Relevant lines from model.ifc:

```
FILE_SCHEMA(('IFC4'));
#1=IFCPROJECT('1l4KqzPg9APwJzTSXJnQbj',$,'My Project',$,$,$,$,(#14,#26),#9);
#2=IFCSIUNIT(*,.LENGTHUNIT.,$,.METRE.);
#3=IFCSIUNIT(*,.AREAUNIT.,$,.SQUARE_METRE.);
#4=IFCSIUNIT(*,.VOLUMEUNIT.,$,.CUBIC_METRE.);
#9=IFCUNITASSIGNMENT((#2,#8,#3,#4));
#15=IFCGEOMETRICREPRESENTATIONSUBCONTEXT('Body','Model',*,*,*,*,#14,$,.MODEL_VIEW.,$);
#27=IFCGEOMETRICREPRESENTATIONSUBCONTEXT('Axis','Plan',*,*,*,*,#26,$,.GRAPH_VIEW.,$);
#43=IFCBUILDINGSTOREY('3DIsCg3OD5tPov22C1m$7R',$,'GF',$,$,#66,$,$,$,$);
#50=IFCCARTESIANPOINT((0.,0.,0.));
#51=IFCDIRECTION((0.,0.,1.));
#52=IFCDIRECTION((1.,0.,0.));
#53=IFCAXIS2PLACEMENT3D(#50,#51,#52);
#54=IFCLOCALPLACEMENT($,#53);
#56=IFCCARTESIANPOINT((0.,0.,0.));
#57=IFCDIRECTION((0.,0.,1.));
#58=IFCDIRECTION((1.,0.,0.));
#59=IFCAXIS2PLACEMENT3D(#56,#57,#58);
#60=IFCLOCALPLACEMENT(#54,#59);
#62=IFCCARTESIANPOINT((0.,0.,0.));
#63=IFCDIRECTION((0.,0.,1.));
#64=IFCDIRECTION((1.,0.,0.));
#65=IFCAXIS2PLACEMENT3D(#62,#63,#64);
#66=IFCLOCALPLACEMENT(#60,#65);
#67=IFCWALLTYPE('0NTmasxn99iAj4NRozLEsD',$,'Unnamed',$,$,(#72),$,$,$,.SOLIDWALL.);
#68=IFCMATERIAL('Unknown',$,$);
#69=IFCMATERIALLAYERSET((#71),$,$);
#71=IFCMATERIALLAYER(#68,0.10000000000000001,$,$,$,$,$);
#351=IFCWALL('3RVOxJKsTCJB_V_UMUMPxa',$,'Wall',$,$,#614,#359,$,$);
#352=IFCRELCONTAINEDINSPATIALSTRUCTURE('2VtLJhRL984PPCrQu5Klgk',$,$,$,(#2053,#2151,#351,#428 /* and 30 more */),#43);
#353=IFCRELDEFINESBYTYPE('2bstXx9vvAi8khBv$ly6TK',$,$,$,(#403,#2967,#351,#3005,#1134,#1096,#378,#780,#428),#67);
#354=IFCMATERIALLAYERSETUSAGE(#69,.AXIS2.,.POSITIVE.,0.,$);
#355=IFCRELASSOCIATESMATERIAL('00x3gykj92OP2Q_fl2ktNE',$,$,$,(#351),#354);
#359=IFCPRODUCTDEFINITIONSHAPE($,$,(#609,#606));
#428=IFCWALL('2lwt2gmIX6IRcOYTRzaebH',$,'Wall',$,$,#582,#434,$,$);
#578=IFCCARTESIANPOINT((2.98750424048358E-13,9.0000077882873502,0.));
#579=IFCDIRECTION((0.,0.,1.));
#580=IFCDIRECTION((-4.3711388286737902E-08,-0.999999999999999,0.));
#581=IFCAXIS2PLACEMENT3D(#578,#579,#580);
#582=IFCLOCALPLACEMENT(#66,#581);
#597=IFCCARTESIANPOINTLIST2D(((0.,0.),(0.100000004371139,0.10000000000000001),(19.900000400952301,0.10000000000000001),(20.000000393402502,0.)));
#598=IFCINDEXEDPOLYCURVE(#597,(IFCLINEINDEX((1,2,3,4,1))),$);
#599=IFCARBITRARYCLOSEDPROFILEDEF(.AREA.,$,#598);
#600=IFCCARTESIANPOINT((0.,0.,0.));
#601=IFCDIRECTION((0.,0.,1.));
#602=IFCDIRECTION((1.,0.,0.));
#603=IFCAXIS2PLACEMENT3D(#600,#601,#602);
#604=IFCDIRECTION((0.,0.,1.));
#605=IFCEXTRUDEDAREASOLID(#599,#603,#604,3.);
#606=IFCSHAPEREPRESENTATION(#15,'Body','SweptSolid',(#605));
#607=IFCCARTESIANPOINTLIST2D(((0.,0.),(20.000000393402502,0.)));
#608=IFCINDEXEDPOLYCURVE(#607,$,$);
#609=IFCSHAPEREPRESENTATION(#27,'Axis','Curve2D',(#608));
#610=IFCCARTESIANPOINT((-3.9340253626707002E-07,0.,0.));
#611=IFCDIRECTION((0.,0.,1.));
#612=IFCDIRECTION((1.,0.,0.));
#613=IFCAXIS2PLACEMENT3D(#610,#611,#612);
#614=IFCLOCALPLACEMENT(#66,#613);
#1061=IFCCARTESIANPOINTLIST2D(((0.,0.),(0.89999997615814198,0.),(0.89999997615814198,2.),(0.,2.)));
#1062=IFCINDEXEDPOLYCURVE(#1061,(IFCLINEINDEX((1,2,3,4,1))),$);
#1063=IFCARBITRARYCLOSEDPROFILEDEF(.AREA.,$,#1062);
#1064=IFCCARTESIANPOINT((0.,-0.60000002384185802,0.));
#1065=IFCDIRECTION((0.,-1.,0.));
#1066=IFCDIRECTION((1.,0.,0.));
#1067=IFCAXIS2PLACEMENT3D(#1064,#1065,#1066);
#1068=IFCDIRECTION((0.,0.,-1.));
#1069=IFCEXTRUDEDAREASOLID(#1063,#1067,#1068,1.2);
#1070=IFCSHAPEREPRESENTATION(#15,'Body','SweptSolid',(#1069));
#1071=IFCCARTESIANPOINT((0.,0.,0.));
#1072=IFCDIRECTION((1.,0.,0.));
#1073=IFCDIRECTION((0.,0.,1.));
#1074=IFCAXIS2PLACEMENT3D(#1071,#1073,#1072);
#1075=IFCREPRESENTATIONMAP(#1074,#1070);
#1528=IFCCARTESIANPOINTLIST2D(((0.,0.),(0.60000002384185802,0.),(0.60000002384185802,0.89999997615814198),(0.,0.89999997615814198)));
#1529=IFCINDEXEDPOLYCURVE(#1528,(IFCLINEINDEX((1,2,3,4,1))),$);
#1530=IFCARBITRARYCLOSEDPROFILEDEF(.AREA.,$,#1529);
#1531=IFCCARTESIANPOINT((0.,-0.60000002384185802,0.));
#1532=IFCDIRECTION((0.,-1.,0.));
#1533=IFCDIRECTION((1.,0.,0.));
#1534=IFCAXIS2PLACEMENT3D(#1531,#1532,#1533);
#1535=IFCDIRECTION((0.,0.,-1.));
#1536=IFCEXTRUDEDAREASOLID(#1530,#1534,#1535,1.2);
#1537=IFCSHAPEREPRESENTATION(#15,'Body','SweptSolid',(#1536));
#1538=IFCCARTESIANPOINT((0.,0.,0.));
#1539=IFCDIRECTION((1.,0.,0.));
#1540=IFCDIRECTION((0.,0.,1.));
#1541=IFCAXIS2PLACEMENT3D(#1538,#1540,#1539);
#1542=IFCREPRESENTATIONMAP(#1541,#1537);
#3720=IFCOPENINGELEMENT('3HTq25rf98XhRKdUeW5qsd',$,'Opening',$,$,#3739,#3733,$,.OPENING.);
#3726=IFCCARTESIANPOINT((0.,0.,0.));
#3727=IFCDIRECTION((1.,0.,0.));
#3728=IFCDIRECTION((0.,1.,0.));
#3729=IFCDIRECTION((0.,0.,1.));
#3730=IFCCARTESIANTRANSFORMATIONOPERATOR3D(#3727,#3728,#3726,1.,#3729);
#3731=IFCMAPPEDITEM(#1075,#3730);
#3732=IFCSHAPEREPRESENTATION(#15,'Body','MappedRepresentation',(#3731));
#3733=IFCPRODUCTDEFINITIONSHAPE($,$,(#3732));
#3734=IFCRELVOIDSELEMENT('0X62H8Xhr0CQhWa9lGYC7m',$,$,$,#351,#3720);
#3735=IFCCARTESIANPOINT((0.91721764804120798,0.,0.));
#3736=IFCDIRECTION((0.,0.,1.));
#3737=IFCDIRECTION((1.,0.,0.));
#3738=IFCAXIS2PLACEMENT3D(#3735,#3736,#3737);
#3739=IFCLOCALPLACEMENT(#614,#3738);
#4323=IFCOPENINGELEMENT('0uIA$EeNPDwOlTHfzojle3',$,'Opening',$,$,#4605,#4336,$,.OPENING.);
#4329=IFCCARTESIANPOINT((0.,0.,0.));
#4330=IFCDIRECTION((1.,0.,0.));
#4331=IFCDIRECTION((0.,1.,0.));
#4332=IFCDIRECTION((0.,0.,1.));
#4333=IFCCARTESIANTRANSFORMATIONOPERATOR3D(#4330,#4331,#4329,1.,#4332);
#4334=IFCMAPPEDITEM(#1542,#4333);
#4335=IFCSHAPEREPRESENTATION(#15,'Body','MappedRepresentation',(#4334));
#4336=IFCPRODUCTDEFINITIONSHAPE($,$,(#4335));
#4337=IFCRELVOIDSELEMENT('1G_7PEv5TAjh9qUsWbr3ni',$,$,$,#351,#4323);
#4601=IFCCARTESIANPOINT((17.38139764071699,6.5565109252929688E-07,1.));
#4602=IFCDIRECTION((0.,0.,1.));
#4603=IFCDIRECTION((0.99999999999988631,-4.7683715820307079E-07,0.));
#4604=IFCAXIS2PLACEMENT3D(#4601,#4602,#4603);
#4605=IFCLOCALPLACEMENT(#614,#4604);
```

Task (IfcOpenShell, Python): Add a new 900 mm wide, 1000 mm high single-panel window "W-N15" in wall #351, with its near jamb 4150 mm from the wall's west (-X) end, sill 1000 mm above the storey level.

```python
import numpy as np
import ifcopenshell
import ifcopenshell.api.feature
import ifcopenshell.api.geometry
import ifcopenshell.api.root
import ifcopenshell.api.spatial
import ifcopenshell.geom
import ifcopenshell.util.element
import ifcopenshell.util.placement
import ifcopenshell.util.representation
import ifcopenshell.util.shape
import ifcopenshell.util.unit

model = ifcopenshell.open("model.ifc")
unit_scale = ifcopenshell.util.unit.calculate_unit_scale(model)
settings = ifcopenshell.geom.settings()


def volume(element):
    """Net volume in cubic metres, openings subtracted."""
    shape = ifcopenshell.geom.create_shape(settings, element)
    return ifcopenshell.util.shape.get_volume(shape.geometry)


wall = model.by_guid("3RVOxJKsTCJB_V_UMUMPxa")
storey = ifcopenshell.util.element.get_container(wall, ifc_class="IfcBuildingStorey")
context = ifcopenshell.util.representation.get_context(model, "Model", "Body", "MODEL_VIEW")
before = volume(wall)

width, height, from_end, sill = 0.9, 1, 4.15, 1  # metres

# The wall runs along its own X axis, and the end named is its -X end.
wall_shape = ifcopenshell.geom.create_shape(settings, wall)
x, y, z = ifcopenshell.util.shape.get_vertices(wall_shape.geometry).T
start = x.min() + from_end
face, thickness = float(y.min()), float(y.max() - y.min())
wall_matrix = ifcopenshell.util.placement.get_local_placement(wall.ObjectPlacement)
level = ifcopenshell.util.placement.get_local_placement(storey.ObjectPlacement)[2, 3]


def in_wall(x, y):
    """Placement at x, y metres in the wall's axes, at sill height."""
    matrix = wall_matrix.copy()
    matrix[:, 3] = wall_matrix @ np.array([x / unit_scale, y / unit_scale, 0.0, 1.0])
    matrix[2, 3] = level + sill / unit_scale
    return matrix


# Opening: a box that overshoots both wall faces by 50 mm.
opening = ifcopenshell.api.root.create_entity(model, ifc_class="IfcOpeningElement", predefined_type="OPENING")
box = ifcopenshell.api.geometry.add_wall_representation(
    model, context=context, length=width, height=height, thickness=thickness + 0.1
)
ifcopenshell.api.geometry.assign_representation(model, product=opening, representation=box)
ifcopenshell.api.geometry.edit_object_placement(model, product=opening, matrix=in_wall(start, face - 0.05), is_si=False)
ifcopenshell.api.feature.add_feature(model, feature=opening, element=wall)

window = ifcopenshell.api.root.create_entity(model, ifc_class="IfcWindow", name="W-N15", predefined_type="WINDOW")
window.OverallWidth, window.OverallHeight = width / unit_scale, height / unit_scale
window.PartitioningType = "SINGLE_PANEL"
body = ifcopenshell.api.geometry.add_window_representation(
    model,
    context=context,
    overall_width=window.OverallWidth,
    overall_height=window.OverallHeight,
    partition_type="SINGLE_PANEL",
)
ifcopenshell.api.geometry.assign_representation(model, product=window, representation=body)
ifcopenshell.api.spatial.assign_container(model, products=[window], relating_structure=storey)
ifcopenshell.api.feature.add_filling(model, opening=opening, element=window)

# Centre the window in the wall's thickness.
ifcopenshell.api.geometry.edit_object_placement(model, product=window, matrix=in_wall(start, face), is_si=False)
window_shape = ifcopenshell.geom.create_shape(settings, window)
depth = ifcopenshell.util.shape.get_vertices(window_shape.geometry)[:, 1]
offset = face + thickness / 2 - (depth.min() + depth.max()) / 2
ifcopenshell.api.geometry.edit_object_placement(model, product=window, matrix=in_wall(start, offset), is_si=False)

after = volume(wall)

print(f"wall volume {before:.3f} -> {after:.3f} m3")

model.write("model_rev.ifc")
```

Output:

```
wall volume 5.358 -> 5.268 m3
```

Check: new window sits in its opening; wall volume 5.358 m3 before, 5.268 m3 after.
